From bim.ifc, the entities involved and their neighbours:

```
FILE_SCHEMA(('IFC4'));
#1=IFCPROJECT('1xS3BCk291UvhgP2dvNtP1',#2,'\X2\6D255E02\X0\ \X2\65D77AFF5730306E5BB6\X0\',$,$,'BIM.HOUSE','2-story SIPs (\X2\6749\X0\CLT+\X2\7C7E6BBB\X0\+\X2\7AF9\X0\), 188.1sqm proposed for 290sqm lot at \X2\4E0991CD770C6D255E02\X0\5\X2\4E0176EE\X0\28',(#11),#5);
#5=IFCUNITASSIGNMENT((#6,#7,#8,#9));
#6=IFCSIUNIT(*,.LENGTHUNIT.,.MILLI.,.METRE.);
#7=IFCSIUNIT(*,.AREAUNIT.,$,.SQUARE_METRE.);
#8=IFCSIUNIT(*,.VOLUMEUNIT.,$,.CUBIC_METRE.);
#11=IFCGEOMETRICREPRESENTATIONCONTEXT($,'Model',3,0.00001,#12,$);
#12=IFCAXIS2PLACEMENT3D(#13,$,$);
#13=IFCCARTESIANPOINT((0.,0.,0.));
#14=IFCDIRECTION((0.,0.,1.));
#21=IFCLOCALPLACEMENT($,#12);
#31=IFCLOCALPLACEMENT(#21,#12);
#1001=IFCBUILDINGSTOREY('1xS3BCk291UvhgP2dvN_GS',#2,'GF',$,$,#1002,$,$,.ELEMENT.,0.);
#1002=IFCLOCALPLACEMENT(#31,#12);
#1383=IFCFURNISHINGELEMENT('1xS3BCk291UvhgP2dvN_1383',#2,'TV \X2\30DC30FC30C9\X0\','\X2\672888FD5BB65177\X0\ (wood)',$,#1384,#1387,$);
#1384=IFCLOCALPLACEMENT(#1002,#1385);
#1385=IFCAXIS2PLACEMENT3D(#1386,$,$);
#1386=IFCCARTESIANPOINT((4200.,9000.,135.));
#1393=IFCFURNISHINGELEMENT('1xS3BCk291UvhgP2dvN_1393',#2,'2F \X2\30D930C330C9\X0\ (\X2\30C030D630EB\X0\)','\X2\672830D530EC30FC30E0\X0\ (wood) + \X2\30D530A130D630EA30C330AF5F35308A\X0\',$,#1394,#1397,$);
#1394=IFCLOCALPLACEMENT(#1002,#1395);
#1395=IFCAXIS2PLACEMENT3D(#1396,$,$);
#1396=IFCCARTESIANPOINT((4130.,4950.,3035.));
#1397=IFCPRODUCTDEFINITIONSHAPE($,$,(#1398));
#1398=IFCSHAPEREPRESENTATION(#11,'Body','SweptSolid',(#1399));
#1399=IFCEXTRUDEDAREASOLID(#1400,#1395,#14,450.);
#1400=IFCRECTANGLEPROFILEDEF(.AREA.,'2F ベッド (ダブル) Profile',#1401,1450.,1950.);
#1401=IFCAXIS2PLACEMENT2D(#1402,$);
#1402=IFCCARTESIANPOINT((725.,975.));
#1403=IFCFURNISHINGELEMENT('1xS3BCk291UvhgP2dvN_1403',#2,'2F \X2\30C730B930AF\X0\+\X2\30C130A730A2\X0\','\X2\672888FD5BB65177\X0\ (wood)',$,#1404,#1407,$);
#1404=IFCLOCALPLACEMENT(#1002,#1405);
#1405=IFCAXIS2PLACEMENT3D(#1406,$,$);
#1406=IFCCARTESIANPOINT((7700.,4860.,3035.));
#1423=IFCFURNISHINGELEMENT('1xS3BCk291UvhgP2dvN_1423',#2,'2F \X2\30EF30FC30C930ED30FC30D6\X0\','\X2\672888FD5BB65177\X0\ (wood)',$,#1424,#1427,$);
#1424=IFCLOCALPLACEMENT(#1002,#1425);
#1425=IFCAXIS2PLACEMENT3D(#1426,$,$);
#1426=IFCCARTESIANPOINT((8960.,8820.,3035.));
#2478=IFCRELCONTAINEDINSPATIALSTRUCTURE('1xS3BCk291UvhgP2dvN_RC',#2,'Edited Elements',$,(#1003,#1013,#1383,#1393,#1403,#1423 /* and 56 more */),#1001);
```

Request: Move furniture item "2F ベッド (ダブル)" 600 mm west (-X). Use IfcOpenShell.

```python
import ifcopenshell
import ifcopenshell.api.geometry
import ifcopenshell.util.placement

model = ifcopenshell.open("bim.ifc")

item = model.by_guid("1xS3BCk291UvhgP2dvN_1393")
matrix = ifcopenshell.util.placement.get_local_placement(item.ObjectPlacement)
matrix[0, 3] -= 600.0
ifcopenshell.api.geometry.edit_object_placement(model, product=item, matrix=matrix, is_si=False)

print(ifcopenshell.util.placement.get_local_placement(item.ObjectPlacement).round(3) + 0.0)

model.write("bim_updated.ifc")
```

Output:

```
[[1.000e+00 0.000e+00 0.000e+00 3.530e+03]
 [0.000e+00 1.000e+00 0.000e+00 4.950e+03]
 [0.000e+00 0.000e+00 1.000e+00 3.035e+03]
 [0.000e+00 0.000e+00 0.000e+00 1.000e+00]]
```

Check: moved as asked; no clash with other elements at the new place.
